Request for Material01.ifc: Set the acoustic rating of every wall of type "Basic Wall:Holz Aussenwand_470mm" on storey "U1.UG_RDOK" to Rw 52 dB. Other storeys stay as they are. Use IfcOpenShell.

First a look at what the model holds.

```python
import ifcopenshell
import ifcopenshell.util.element

model = ifcopenshell.open("Material01.ifc")
print(model.schema)
storey = next(s for s in model.by_type("IfcBuildingStorey") if s.Name == "U1.UG_RDOK")
walls = [e for e in ifcopenshell.util.element.get_decomposition(storey) if e.is_a("IfcWall")]
seen = {}
for e in walls:
    element_type = ifcopenshell.util.element.get_type(e)
    key = (element_type.Name if element_type != e and element_type else None, ifcopenshell.util.element.get_pset(e, "Pset_WallCommon", "AcousticRating"))
    seen[key] = seen.get(key, 0) + 1
for (name, value), count in sorted(seen.items(), key=str):
    print(count, "x", name, "|", value)
```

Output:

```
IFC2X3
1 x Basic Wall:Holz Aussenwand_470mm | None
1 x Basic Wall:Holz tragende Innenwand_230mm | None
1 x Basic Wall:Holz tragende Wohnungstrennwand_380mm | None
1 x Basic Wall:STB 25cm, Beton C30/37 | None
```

```python
import ifcopenshell
import ifcopenshell.api.pset
import ifcopenshell.util.element

model = ifcopenshell.open("Material01.ifc")

storey = next(s for s in model.by_type("IfcBuildingStorey") if s.Name == "U1.UG_RDOK")
walls = [e for e in ifcopenshell.util.element.get_decomposition(storey) if e.is_a("IfcWall")]

count = 0
for e in walls:
    element_type = ifcopenshell.util.element.get_type(e)
    if element_type in (None, e) or element_type.Name != "Basic Wall:Holz Aussenwand_470mm":
        continue
    # add_pset returns the element's existing set when there is one.
    pset = ifcopenshell.api.pset.add_pset(model, product=e, name="Pset_WallCommon")
    ifcopenshell.api.pset.edit_pset(model, pset=pset, properties={"AcousticRating": "Rw 52 dB"})
    count += 1

print(count, "walls updated")

model.write("Material01_updated.ifc")
```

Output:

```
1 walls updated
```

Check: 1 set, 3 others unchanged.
